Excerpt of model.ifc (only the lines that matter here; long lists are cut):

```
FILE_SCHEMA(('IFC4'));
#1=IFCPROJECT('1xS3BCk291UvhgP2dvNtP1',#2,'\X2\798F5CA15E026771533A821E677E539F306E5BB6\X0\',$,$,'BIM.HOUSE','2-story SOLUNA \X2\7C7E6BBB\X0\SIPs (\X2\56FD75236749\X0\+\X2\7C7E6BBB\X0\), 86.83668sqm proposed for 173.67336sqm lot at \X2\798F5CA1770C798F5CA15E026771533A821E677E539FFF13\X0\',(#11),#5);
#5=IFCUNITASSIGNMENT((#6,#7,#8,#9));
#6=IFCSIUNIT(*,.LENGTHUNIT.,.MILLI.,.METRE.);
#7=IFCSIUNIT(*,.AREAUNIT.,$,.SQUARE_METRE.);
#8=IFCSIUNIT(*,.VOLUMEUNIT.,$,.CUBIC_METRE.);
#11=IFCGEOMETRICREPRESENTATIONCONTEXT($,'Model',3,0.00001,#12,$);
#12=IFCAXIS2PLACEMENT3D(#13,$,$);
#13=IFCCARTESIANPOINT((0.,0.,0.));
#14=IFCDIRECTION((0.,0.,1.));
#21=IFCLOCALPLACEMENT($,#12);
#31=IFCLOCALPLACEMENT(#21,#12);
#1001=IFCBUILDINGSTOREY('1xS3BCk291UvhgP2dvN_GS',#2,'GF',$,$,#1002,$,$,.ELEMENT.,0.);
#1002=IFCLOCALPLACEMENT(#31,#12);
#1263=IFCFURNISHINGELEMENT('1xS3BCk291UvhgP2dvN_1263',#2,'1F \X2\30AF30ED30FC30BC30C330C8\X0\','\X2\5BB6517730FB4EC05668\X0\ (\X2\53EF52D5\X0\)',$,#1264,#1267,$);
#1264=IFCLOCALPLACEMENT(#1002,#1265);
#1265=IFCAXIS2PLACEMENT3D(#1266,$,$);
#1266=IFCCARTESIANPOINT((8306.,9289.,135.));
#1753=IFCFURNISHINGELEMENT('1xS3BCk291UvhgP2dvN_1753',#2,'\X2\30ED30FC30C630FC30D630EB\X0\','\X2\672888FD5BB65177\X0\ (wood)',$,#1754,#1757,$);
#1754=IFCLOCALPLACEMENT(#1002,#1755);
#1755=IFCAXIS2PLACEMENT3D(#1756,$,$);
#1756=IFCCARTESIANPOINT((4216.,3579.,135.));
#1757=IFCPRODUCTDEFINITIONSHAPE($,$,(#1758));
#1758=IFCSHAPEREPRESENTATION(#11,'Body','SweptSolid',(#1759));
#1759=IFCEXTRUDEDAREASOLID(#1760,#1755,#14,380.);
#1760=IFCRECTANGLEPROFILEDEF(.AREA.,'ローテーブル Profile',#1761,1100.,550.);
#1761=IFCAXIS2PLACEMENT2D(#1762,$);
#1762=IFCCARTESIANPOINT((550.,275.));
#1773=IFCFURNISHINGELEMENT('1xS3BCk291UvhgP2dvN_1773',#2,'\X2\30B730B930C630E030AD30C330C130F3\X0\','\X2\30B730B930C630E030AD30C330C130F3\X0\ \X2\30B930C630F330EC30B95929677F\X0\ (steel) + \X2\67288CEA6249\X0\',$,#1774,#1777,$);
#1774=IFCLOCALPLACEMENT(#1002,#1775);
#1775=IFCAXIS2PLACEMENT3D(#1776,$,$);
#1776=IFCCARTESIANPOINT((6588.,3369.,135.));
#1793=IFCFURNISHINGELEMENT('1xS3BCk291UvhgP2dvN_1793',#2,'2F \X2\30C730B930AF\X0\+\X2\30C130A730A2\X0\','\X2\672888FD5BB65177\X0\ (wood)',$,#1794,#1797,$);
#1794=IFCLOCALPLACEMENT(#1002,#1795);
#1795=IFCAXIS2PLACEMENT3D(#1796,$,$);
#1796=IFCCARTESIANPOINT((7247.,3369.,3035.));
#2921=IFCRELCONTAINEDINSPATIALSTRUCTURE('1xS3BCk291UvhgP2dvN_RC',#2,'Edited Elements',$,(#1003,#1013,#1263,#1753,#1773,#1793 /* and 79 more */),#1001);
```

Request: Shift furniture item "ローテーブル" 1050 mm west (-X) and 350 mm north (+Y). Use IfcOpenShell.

```python
import ifcopenshell
import ifcopenshell.api.geometry
import ifcopenshell.util.placement

model = ifcopenshell.open("model.ifc")

item = model.by_id(1753)
matrix = ifcopenshell.util.placement.get_local_placement(item.ObjectPlacement)
matrix[0, 3] -= 1050.0
matrix[1, 3] += 350.0
ifcopenshell.api.geometry.edit_object_placement(model, product=item, matrix=matrix, is_si=False)

print(ifcopenshell.util.placement.get_local_placement(item.ObjectPlacement).round(3) + 0.0)

model.write("model_updated.ifc")
```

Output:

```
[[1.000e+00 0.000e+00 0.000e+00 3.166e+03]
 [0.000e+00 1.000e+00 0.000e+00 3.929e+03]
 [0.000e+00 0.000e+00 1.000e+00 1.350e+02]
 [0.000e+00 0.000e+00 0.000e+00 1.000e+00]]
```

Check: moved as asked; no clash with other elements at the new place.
